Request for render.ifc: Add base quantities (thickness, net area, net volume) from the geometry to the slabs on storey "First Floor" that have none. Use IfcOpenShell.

First a look at what the model holds.

```python
import ifcopenshell
import ifcopenshell.util.element
import ifcopenshell.util.unit

model = ifcopenshell.open("render.ifc")
print(model.schema)
for unit_type in ("LENGTHUNIT", "AREAUNIT", "VOLUMEUNIT"):
    print(unit_type, ifcopenshell.util.unit.calculate_unit_scale(model, unit_type))
storey = next(s for s in model.by_type("IfcBuildingStorey") if s.Name == "First Floor")
slabs = [e for e in ifcopenshell.util.element.get_decomposition(storey) if e.is_a("IfcSlab")]
for e in sorted(slabs, key=lambda e: e.id()):
    print(e.id(), e.is_a(), e.Name, list(ifcopenshell.util.element.get_psets(e, qtos_only=True)), sep=" | ")
```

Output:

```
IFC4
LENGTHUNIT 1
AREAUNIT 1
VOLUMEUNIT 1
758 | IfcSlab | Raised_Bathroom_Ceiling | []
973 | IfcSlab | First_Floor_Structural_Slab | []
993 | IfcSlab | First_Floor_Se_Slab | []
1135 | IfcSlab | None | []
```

```python
import ifcopenshell
import ifcopenshell.api.pset
import ifcopenshell.geom
import ifcopenshell.util.element
import ifcopenshell.util.shape
import ifcopenshell.util.unit

model = ifcopenshell.open("render.ifc")
unit_scale = ifcopenshell.util.unit.calculate_unit_scale(model)
area_scale = ifcopenshell.util.unit.calculate_unit_scale(model, "AREAUNIT")
volume_scale = ifcopenshell.util.unit.calculate_unit_scale(model, "VOLUMEUNIT")
settings = ifcopenshell.geom.settings()

storey = next(s for s in model.by_type("IfcBuildingStorey") if s.Name == "First Floor")
slabs = [e for e in ifcopenshell.util.element.get_decomposition(storey) if e.is_a("IfcSlab")]

for e in sorted(slabs, key=lambda e: e.id()):
    if ifcopenshell.util.element.get_psets(e, qtos_only=True, should_inherit=False):
        continue
    # Geometry comes back in metres, in the element's own axes.
    shape = ifcopenshell.geom.create_shape(settings, e)
    values = {
        "Width": ifcopenshell.util.shape.get_z(shape.geometry) / unit_scale,
        "NetArea": ifcopenshell.util.shape.get_footprint_area(shape.geometry) / area_scale,
        "NetVolume": ifcopenshell.util.shape.get_volume(shape.geometry) / volume_scale,
    }
    qto = ifcopenshell.api.pset.add_qto(model, product=e, name="Qto_SlabBaseQuantities")
    ifcopenshell.api.pset.edit_qto(model, qto=qto, properties=values)
    print(e.id(), {k: round(v, 3) for k, v in values.items()})

model.write("render_v2.ifc")
```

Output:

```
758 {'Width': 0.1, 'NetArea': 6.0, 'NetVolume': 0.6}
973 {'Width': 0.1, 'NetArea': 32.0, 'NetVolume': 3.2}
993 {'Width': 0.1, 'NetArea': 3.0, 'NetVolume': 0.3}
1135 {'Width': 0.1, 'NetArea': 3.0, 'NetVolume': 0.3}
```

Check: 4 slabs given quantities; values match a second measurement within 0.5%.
